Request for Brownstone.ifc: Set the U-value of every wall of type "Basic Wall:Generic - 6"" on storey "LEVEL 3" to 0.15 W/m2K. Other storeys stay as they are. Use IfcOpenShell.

First a look at what the model holds.

```python
import ifcopenshell
import ifcopenshell.util.element

model = ifcopenshell.open("Brownstone.ifc")
print(model.schema)
storey = next(s for s in model.by_type("IfcBuildingStorey") if s.Name == "LEVEL 3")
walls = [e for e in ifcopenshell.util.element.get_decomposition(storey) if e.is_a("IfcWall")]
seen = {}
for e in walls:
    element_type = ifcopenshell.util.element.get_type(e)
    key = (element_type.Name if element_type != e and element_type else None, ifcopenshell.util.element.get_pset(e, "Pset_WallCommon", "ThermalTransmittance"))
    seen[key] = seen.get(key, 0) + 1
for (name, value), count in sorted(seen.items(), key=str):
    print(count, "x", name, "|", value)
```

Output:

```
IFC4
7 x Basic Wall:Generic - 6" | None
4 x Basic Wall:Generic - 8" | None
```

```python
import ifcopenshell
import ifcopenshell.api.pset
import ifcopenshell.util.element

model = ifcopenshell.open("Brownstone.ifc")

storey = next(s for s in model.by_type("IfcBuildingStorey") if s.Name == "LEVEL 3")
walls = [e for e in ifcopenshell.util.element.get_decomposition(storey) if e.is_a("IfcWall")]

count = 0
for e in walls:
    element_type = ifcopenshell.util.element.get_type(e)
    if element_type in (None, e) or element_type.Name != 'Basic Wall:Generic - 6"':
        continue
    # add_pset returns the element's existing set when there is one.
    pset = ifcopenshell.api.pset.add_pset(model, product=e, name="Pset_WallCommon")
    ifcopenshell.api.pset.edit_pset(model, pset=pset, properties={"ThermalTransmittance": 0.15})
    count += 1

print(count, "walls updated")

model.write("Brownstone_rev.ifc")
```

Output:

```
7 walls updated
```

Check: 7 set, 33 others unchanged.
